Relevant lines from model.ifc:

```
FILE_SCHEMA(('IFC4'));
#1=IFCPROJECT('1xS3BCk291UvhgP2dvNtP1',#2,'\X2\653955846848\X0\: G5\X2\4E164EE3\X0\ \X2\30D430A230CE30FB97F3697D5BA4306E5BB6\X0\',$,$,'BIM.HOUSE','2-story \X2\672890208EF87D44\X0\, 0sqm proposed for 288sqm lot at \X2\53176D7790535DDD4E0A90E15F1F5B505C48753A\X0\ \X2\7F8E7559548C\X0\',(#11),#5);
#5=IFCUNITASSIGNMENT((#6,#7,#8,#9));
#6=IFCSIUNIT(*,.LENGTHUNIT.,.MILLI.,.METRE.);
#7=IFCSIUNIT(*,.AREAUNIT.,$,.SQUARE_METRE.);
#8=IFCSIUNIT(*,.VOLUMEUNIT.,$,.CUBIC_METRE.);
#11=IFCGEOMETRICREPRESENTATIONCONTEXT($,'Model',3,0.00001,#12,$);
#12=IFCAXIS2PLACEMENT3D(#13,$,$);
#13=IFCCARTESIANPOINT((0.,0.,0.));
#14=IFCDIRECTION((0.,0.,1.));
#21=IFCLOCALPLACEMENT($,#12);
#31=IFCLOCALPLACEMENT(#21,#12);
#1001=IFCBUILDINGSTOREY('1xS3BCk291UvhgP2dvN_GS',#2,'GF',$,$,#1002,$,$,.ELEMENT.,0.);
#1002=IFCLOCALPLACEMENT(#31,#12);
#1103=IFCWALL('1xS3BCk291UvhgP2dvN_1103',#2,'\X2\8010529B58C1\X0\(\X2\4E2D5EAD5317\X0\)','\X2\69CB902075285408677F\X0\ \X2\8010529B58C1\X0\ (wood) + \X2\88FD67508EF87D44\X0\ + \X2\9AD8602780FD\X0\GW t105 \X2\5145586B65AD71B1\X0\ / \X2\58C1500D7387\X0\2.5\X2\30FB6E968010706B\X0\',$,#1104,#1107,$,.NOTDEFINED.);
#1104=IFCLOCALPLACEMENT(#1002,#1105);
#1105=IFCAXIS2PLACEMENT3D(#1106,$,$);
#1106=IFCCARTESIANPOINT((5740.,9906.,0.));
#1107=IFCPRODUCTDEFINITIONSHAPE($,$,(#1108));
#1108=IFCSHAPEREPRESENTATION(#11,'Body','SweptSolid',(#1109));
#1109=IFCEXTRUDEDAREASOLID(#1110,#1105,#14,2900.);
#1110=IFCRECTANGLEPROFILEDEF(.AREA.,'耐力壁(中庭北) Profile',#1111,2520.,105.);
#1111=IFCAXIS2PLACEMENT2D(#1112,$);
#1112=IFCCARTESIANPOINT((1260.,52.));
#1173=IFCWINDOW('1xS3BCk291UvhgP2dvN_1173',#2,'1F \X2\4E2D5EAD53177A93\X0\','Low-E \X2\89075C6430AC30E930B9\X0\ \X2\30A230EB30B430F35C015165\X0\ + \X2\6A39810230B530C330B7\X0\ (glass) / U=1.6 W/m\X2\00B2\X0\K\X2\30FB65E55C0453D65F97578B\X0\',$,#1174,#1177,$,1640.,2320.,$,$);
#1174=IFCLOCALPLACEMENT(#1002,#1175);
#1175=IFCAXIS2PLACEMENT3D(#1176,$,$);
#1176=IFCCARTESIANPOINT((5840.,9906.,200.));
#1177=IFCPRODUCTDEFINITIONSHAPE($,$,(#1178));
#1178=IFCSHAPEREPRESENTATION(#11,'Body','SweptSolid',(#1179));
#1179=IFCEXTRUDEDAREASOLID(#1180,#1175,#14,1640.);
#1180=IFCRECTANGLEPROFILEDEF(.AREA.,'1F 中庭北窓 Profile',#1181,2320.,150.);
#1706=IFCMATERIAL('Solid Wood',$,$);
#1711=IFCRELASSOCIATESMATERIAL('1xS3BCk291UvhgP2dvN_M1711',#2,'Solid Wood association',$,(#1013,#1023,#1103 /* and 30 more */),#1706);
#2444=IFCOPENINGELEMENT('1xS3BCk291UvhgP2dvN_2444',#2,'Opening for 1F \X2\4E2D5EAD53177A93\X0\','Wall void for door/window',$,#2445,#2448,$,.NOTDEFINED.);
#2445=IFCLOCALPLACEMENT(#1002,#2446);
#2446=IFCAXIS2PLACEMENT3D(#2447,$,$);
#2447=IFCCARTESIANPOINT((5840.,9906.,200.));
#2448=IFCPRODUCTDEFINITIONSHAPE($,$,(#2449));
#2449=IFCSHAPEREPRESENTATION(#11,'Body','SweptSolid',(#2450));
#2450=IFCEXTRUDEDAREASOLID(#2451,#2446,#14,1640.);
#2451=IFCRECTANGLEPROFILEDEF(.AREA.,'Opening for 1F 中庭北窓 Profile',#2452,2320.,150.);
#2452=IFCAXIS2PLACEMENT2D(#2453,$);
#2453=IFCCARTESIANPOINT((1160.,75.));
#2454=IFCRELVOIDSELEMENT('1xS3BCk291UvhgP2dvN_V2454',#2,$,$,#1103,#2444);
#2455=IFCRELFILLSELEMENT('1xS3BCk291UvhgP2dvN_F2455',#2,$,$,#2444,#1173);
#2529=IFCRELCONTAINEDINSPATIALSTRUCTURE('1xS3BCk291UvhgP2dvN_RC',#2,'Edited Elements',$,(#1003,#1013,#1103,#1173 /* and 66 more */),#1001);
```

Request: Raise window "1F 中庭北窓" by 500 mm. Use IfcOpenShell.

```python
import numpy as np
import ifcopenshell
import ifcopenshell.api.geometry
import ifcopenshell.util.placement
import ifcopenshell.util.unit

model = ifcopenshell.open("model.ifc")
unit_scale = ifcopenshell.util.unit.calculate_unit_scale(model)

window = model.by_guid("1xS3BCk291UvhgP2dvN_1173")
opening = window.FillsVoids[0].RelatingOpeningElement
dz = 500.0

shift = np.array([0.0, 0.0, dz])
# The window is not placed relative to its opening, so move both.
for product in (opening, window):
    matrix = ifcopenshell.util.placement.get_local_placement(product.ObjectPlacement)
    matrix[:3, 3] += shift
    ifcopenshell.api.geometry.edit_object_placement(model, product=product, matrix=matrix, is_si=False)

print(f"moved by {dz * unit_scale:+.3f} m")

model.write("model_rev.ifc")
```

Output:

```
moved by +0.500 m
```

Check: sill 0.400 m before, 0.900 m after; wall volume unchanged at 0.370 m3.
